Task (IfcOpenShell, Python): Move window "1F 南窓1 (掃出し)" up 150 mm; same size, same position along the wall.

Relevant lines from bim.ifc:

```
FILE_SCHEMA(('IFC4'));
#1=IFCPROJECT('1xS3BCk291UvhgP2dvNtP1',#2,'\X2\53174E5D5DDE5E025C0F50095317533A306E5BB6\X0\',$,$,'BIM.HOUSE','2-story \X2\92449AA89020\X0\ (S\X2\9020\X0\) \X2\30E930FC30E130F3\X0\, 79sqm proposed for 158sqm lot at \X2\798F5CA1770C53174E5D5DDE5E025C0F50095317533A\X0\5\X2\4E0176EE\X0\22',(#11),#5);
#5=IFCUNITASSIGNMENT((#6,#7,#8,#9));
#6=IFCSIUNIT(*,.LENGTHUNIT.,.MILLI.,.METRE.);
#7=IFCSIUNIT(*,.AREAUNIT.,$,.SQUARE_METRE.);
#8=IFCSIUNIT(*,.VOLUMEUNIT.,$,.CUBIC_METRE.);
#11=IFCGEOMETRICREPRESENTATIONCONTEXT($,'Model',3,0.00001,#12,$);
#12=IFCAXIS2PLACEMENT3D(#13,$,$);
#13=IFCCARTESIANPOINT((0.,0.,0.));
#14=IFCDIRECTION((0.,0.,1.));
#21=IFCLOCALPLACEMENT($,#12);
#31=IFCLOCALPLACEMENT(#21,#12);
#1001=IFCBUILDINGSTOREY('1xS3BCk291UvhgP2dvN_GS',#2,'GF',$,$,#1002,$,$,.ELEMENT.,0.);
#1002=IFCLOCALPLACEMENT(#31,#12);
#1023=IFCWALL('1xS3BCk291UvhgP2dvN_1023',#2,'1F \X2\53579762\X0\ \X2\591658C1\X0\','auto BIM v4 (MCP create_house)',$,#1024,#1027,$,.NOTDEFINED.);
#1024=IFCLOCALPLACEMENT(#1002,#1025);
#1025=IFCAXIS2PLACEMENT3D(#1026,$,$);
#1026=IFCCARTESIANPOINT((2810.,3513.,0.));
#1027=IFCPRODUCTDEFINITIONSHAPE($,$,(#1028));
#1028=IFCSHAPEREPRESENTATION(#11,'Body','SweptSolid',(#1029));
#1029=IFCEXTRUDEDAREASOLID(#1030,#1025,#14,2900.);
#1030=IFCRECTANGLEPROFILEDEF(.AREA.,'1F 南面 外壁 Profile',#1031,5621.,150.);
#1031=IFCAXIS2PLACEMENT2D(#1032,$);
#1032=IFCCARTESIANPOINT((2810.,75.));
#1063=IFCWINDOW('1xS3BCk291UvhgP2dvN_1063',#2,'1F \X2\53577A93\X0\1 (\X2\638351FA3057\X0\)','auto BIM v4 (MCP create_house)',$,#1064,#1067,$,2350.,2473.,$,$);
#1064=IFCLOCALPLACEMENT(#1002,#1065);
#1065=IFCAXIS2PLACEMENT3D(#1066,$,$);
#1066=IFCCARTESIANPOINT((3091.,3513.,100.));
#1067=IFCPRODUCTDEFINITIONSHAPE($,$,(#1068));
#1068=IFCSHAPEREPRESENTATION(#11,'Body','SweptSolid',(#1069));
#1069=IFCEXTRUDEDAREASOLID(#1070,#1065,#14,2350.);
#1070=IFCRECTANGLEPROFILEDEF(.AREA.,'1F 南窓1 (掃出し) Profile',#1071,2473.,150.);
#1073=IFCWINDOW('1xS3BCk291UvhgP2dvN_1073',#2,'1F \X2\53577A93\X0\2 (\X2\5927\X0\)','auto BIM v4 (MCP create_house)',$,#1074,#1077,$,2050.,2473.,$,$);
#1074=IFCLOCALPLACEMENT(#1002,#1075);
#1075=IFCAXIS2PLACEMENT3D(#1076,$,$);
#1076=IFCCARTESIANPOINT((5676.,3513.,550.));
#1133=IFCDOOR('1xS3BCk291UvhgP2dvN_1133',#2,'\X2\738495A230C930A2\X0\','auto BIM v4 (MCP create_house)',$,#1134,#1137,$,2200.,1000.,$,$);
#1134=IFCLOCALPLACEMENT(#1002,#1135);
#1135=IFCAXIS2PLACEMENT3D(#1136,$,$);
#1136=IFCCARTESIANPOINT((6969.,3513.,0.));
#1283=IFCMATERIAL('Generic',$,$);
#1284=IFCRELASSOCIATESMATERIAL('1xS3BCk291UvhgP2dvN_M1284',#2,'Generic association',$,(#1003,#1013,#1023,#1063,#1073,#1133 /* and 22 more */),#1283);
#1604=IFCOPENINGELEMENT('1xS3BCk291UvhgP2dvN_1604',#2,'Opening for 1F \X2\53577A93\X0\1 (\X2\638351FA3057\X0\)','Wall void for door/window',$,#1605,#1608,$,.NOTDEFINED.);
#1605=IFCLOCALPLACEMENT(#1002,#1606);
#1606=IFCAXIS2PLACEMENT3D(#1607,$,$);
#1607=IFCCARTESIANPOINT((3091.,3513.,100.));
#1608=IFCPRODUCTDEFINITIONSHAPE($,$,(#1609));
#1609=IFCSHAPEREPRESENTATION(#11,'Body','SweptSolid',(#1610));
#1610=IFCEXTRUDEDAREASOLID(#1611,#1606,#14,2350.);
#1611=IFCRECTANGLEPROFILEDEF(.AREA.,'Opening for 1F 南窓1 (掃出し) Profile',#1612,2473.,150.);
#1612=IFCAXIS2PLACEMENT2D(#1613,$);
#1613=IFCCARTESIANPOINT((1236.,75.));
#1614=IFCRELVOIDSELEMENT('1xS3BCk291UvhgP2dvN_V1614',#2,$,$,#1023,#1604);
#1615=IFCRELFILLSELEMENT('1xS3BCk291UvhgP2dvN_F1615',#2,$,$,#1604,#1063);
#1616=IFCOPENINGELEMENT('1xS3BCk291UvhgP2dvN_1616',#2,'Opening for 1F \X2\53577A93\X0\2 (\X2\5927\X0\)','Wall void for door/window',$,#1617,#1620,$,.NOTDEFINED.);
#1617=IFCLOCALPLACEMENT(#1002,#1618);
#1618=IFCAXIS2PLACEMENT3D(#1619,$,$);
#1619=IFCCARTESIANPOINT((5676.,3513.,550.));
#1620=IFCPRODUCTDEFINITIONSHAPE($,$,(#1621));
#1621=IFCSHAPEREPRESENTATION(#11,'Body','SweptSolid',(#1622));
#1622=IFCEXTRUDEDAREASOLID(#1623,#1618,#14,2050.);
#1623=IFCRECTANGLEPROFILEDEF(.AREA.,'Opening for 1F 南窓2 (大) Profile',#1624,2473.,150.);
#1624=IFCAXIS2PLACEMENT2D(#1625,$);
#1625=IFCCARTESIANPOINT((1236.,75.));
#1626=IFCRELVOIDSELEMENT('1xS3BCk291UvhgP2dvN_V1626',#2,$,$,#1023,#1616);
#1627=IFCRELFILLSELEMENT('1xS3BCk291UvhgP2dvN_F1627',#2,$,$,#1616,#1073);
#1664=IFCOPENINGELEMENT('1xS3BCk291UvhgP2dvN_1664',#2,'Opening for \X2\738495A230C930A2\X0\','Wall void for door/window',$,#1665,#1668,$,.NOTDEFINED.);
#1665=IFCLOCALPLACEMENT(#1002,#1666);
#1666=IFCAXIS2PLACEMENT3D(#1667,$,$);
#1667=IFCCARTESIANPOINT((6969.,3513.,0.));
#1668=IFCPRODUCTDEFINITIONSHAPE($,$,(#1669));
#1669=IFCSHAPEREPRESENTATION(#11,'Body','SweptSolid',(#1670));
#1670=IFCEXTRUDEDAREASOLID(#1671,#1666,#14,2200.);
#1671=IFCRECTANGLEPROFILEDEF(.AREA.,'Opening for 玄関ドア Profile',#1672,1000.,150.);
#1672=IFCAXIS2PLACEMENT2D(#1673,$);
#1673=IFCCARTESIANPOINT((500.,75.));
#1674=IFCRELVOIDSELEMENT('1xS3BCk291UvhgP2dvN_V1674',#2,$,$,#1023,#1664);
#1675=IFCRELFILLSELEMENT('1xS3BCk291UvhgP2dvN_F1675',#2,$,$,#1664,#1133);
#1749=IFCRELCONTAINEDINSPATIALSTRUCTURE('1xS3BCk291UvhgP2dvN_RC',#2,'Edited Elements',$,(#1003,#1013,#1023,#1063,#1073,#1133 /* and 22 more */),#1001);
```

```python
import numpy as np
import ifcopenshell
import ifcopenshell.api.geometry
import ifcopenshell.util.placement
import ifcopenshell.util.unit

model = ifcopenshell.open("bim.ifc")
unit_scale = ifcopenshell.util.unit.calculate_unit_scale(model)

window = model.by_guid("1xS3BCk291UvhgP2dvN_1063")
opening = window.FillsVoids[0].RelatingOpeningElement
dz = 0.15 / unit_scale

shift = np.array([0.0, 0.0, dz])
# The window is not placed relative to its opening, so move both.
for product in (opening, window):
    matrix = ifcopenshell.util.placement.get_local_placement(product.ObjectPlacement)
    matrix[:3, 3] += shift
    ifcopenshell.api.geometry.edit_object_placement(model, product=product, matrix=matrix, is_si=False)

print(f"moved by {dz * unit_scale:+.3f} m")

model.write("bim-out.ifc")
```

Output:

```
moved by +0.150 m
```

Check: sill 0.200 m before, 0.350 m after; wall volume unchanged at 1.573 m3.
